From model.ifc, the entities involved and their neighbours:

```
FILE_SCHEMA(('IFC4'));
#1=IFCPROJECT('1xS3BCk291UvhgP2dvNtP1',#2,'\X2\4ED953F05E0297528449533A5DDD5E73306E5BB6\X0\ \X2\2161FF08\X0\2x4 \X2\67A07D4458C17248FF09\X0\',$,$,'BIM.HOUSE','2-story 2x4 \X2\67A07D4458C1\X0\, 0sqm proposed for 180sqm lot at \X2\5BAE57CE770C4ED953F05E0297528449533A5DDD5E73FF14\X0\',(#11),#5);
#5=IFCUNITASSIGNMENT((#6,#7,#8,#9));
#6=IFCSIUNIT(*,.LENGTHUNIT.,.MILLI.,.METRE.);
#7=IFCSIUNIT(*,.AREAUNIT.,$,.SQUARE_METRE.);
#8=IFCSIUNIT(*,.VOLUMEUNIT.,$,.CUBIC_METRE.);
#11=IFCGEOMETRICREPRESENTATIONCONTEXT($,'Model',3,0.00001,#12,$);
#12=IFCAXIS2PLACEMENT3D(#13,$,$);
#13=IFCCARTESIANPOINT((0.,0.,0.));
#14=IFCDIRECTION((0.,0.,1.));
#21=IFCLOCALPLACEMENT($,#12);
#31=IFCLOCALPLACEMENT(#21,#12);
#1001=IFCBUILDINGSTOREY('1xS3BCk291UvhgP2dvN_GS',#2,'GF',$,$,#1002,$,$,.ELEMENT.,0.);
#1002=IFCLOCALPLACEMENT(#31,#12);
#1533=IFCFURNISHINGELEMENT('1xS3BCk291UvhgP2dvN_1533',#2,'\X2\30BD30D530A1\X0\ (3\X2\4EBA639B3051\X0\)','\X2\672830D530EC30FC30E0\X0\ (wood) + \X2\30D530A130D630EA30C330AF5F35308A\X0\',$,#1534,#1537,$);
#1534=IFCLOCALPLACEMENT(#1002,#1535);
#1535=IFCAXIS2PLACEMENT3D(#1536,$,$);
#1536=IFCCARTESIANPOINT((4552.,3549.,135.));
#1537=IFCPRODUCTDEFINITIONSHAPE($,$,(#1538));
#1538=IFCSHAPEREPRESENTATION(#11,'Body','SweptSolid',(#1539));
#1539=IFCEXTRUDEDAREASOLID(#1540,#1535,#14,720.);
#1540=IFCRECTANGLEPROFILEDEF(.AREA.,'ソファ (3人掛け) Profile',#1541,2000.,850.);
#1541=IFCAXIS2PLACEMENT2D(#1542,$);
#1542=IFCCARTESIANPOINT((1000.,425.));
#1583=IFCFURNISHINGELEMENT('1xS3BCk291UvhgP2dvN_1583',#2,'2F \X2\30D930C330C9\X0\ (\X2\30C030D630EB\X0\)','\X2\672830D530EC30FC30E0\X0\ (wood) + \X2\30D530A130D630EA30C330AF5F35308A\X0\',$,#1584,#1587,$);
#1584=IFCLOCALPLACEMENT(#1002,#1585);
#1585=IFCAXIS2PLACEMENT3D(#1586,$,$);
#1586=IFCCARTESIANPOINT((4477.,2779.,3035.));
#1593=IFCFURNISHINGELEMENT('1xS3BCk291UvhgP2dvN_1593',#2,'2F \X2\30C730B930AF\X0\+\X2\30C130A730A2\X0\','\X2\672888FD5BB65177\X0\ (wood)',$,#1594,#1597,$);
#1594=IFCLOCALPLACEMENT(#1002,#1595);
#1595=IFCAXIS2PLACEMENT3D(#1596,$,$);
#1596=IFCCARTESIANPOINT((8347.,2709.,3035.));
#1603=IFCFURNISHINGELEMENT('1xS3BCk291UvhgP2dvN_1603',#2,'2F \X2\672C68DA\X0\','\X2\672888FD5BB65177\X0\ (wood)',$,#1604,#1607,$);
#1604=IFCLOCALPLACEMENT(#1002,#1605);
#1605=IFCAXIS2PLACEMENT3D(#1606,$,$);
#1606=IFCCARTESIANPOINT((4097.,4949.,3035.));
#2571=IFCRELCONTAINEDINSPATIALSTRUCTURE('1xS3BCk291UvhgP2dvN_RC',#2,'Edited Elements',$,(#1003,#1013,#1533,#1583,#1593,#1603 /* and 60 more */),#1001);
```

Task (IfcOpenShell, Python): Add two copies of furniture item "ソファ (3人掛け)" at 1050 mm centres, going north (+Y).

```python
import numpy as np
import ifcopenshell
import ifcopenshell.api.geometry
import ifcopenshell.api.root
import ifcopenshell.util.element
import ifcopenshell.util.placement
import ifcopenshell.util.unit

model = ifcopenshell.open("model.ifc")
unit_scale = ifcopenshell.util.unit.calculate_unit_scale(model)


def reuse_history(source, copy):
    """copy_class also copies each property set's owner history, people and application; keep the originals."""
    for rel in copy.IsDefinedBy:
        if rel.is_a("IfcRelDefinesByProperties") and (history := rel.RelatingPropertyDefinition.OwnerHistory):
            rel.RelatingPropertyDefinition.OwnerHistory = source.OwnerHistory
            ifcopenshell.util.element.remove_deep2(model, history)


source = model.by_id(1533)
base = ifcopenshell.util.placement.get_local_placement(source.ObjectPlacement)
step = np.array([0.0, 1.0, 0.0]) * 1.05 / unit_scale

for i in range(1, 3):
    copy = ifcopenshell.api.root.copy_class(model, product=source)
    copy.Representation = ifcopenshell.util.element.copy_deep(
        model, source.Representation, exclude=["IfcGeometricRepresentationContext", "IfcRepresentationMap"]
    )
    reuse_history(source, copy)
    matrix = base.copy()
    matrix[:3, 3] += i * step
    print("added at", matrix[:3, 3].round(3) + 0.0)
    ifcopenshell.api.geometry.edit_object_placement(model, product=copy, matrix=matrix, is_si=False)

model.write("model_updated.ifc")
```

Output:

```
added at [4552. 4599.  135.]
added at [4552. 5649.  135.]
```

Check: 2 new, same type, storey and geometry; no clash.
